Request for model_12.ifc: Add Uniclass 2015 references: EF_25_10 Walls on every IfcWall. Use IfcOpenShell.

First a look at what the model holds.

```python
import ifcopenshell

model = ifcopenshell.open("model_12.ifc")
print(model.schema)
print("classifications:", [c.Name for c in model.by_type("IfcClassification")])
for ifc_class in ("IfcDoor", "IfcRoof", "IfcStair", "IfcWall", "IfcWindow"):
    print(ifc_class, len(model.by_type(ifc_class)))
```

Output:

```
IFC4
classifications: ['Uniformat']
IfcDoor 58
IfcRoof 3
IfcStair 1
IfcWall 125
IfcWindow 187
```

```python
import ifcopenshell
import ifcopenshell.api.classification

model = ifcopenshell.open("model_12.ifc")

system = ifcopenshell.api.classification.add_classification(model, classification="Uniclass 2015")

codes = {
    "IfcWall": ("EF_25_10", "Walls"),
}
for ifc_class, (code, name) in codes.items():
    products = model.by_type(ifc_class)
    ifcopenshell.api.classification.add_reference(
        model, products=products, classification=system, identification=code, name=name
    )
    print(code, len(products))

model.write("model_12_v2.ifc")
```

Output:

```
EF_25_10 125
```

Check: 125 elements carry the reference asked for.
